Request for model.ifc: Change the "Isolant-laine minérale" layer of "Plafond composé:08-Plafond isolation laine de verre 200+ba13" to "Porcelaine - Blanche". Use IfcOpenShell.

First a look at what the model holds.

```python
import ifcopenshell
import ifcopenshell.util.element

model = ifcopenshell.open("model.ifc")
print(model.schema)
for layer_set in model.by_type("IfcMaterialLayerSet"):
    if layer_set.LayerSetName == "Plafond composé:08-Plafond isolation laine de verre 200+ba13":
        for layer in layer_set.MaterialLayers:
            print(layer.id(), layer.Material and layer.Material.Name, layer.LayerThickness, sep=" | ")
        print(len(ifcopenshell.util.element.get_elements_by_material(model, layer_set)), "elements and types use it")
print(sorted(m.Name for m in model.by_type("IfcMaterial") if m.Name)[:60])
```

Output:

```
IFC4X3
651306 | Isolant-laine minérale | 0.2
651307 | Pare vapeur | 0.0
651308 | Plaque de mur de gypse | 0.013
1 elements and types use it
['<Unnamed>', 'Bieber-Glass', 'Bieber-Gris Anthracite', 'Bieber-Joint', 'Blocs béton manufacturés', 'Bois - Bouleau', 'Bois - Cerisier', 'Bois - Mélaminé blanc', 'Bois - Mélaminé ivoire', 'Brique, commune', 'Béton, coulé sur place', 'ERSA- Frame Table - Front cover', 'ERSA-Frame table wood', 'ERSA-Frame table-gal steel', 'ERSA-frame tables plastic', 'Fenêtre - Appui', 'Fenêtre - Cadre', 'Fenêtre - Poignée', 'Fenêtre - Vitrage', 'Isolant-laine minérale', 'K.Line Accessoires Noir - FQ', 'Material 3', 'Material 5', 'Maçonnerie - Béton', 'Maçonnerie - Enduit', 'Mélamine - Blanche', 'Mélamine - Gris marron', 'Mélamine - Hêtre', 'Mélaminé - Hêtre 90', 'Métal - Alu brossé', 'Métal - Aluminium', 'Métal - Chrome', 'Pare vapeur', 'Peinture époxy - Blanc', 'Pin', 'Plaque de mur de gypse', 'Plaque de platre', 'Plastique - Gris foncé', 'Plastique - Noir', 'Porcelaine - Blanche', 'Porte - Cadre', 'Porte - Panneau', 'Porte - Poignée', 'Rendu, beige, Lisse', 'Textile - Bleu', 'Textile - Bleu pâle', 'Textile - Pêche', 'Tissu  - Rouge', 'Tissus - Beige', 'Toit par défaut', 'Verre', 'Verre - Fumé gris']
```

```python
import ifcopenshell
import ifcopenshell.api.material

model = ifcopenshell.open("model.ifc")

layer_set = next(s for s in model.by_type("IfcMaterialLayerSet") if s.LayerSetName == "Plafond composé:08-Plafond isolation laine de verre 200+ba13")
layer = next(l for l in layer_set.MaterialLayers if l.Material and l.Material.Name == "Isolant-laine minérale")
material = next(m for m in model.by_type("IfcMaterial") if m.Name == "Porcelaine - Blanche")

# Point this one layer at the other material; renaming the old one would change it everywhere.
ifcopenshell.api.material.edit_layer(model, layer=layer, attributes={"Name": material.Name}, material=material)

print([l.Material.Name if l.Material else None for l in layer_set.MaterialLayers])

model.write("model_v2.ifc")
```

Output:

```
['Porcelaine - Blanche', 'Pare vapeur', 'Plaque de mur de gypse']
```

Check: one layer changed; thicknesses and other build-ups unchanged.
